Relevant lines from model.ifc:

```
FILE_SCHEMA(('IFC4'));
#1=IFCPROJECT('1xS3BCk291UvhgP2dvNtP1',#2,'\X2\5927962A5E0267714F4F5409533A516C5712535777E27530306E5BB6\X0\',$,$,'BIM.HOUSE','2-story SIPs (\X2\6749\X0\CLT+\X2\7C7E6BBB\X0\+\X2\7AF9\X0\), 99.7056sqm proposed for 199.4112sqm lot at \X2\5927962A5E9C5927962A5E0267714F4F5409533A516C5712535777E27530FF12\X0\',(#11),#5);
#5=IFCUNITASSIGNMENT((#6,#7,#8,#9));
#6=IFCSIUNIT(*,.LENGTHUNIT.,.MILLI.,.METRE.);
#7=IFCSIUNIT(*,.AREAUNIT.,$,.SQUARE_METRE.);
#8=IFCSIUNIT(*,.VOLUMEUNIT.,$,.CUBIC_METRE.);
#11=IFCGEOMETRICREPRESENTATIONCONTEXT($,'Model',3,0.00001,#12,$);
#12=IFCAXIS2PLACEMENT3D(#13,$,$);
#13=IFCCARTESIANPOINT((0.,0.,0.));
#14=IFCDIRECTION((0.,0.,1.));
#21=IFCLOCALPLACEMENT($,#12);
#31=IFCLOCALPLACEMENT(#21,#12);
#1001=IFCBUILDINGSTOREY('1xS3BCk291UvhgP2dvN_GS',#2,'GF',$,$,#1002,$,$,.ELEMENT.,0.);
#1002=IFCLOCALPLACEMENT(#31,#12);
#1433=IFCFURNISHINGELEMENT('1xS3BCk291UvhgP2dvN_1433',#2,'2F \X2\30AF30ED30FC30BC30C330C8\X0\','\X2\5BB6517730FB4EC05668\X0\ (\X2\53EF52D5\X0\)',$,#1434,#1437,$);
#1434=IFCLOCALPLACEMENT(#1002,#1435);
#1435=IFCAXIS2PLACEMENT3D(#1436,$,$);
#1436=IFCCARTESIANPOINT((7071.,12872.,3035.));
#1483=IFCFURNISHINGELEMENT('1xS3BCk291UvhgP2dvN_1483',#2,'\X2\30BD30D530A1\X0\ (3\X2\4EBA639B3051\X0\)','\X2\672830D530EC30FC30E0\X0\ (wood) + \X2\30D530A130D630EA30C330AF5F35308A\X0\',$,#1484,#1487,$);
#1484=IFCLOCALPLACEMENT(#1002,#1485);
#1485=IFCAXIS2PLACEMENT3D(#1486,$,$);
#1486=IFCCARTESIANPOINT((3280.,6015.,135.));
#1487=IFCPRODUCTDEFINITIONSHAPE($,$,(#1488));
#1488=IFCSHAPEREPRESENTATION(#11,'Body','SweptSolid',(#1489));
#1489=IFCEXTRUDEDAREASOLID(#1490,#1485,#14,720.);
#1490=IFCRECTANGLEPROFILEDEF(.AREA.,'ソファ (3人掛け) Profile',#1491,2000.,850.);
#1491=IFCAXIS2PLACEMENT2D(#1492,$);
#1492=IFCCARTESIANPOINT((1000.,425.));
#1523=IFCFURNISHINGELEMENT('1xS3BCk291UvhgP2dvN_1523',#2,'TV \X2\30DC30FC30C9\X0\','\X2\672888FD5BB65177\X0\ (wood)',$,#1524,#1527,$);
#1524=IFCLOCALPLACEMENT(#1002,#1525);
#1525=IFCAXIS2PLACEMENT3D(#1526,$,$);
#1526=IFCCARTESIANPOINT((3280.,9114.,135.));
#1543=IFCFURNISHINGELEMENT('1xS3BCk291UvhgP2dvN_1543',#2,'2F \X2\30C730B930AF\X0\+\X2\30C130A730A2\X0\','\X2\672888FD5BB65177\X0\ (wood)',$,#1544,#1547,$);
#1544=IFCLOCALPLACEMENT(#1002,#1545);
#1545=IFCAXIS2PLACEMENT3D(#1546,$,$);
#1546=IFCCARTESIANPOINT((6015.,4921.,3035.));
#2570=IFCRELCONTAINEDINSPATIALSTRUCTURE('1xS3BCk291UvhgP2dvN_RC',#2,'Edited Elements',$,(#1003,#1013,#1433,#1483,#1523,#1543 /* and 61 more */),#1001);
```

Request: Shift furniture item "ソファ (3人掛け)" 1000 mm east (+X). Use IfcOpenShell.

```python
import ifcopenshell
import ifcopenshell.api.geometry
import ifcopenshell.util.placement
import ifcopenshell.util.unit

model = ifcopenshell.open("model.ifc")
unit_scale = ifcopenshell.util.unit.calculate_unit_scale(model)

item = model.by_guid("1xS3BCk291UvhgP2dvN_1483")
matrix = ifcopenshell.util.placement.get_local_placement(item.ObjectPlacement)
matrix[0, 3] += 1 / unit_scale
ifcopenshell.api.geometry.edit_object_placement(model, product=item, matrix=matrix, is_si=False)

print(ifcopenshell.util.placement.get_local_placement(item.ObjectPlacement).round(3) + 0.0)

model.write("model_updated.ifc")
```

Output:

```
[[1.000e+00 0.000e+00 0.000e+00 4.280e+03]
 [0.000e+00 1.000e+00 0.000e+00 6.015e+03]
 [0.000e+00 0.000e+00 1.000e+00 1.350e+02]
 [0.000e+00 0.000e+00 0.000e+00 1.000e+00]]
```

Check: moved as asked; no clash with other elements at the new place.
